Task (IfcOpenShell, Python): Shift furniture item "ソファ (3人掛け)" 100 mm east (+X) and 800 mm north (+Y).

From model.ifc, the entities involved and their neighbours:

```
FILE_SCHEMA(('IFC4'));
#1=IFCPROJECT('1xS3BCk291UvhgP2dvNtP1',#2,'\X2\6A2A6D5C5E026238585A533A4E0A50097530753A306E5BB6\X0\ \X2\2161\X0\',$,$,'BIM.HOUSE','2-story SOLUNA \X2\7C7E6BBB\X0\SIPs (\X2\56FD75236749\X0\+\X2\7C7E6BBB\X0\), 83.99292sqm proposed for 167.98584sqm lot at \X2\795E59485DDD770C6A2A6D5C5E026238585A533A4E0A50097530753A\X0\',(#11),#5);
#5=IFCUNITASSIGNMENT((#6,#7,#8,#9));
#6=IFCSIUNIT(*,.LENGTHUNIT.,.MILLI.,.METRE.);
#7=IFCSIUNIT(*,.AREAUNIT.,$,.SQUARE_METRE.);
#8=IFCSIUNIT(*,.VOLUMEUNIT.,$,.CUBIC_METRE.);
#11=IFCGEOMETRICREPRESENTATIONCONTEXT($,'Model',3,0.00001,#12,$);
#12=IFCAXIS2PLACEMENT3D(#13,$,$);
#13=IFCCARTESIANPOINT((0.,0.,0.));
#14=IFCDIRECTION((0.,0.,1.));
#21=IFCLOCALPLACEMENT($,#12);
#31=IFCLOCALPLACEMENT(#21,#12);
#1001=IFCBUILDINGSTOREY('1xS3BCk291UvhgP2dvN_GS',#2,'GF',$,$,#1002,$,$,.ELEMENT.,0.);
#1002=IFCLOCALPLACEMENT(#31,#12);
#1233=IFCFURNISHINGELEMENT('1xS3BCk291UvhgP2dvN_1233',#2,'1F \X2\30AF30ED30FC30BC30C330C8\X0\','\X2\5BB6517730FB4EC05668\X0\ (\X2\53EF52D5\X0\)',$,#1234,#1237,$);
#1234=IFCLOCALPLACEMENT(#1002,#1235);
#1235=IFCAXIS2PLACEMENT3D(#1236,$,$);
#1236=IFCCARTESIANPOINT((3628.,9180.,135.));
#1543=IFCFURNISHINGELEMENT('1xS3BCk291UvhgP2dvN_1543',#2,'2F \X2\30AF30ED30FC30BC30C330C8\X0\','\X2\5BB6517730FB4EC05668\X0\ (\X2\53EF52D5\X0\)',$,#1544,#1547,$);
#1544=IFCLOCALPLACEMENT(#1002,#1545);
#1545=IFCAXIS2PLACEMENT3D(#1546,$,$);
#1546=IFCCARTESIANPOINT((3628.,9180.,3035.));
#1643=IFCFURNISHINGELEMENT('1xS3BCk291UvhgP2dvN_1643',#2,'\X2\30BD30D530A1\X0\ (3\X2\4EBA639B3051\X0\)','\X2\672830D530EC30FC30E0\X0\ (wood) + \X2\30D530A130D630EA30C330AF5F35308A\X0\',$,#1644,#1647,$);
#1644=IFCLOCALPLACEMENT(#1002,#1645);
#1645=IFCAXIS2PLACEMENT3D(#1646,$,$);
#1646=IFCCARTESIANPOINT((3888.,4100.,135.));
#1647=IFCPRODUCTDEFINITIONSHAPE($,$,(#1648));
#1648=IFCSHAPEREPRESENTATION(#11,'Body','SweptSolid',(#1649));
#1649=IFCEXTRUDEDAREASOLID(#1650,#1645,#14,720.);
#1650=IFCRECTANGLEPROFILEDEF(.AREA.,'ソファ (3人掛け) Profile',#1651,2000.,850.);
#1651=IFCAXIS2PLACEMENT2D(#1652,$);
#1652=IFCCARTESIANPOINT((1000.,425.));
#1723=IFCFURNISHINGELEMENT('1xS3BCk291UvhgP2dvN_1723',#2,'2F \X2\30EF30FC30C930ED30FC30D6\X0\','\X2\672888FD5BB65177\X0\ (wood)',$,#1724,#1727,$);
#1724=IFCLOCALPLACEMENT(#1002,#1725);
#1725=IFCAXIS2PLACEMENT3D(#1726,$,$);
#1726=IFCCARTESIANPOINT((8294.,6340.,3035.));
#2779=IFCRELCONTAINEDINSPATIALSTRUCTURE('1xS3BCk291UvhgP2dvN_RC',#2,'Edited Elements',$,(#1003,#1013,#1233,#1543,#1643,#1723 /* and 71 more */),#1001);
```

```python
import ifcopenshell
import ifcopenshell.api.geometry
import ifcopenshell.util.placement

model = ifcopenshell.open("model.ifc")

item = model.by_id(1643)
matrix = ifcopenshell.util.placement.get_local_placement(item.ObjectPlacement)
matrix[0, 3] += 100.0
matrix[1, 3] += 800.0
ifcopenshell.api.geometry.edit_object_placement(model, product=item, matrix=matrix, is_si=False)

print(ifcopenshell.util.placement.get_local_placement(item.ObjectPlacement).round(3) + 0.0)

model.write("model_v2.ifc")
```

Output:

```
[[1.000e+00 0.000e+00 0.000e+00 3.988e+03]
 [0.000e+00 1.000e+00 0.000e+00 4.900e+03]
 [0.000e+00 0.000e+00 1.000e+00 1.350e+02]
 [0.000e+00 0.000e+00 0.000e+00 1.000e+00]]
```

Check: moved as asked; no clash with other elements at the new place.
